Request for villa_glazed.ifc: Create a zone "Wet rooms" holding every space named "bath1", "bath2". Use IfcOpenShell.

First a look at what the model holds.

```python
import ifcopenshell

model = ifcopenshell.open("villa_glazed.ifc")
print(model.schema)
seen = {}
for space in model.by_type("IfcSpace"):
    seen[space.LongName] = seen.get(space.LongName, 0) + 1
for name, count in sorted(seen.items(), key=str):
    print(count, "x", name)
print("zones:", [z.Name for z in model.by_type("IfcZone")][:20])
```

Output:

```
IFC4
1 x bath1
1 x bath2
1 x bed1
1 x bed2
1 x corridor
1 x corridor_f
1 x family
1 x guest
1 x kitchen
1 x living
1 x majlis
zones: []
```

```python
import ifcopenshell
import ifcopenshell.api.group
import ifcopenshell.api.root

model = ifcopenshell.open("villa_glazed.ifc")

names = {"bath1", "bath2"}
spaces = [s for s in model.by_type("IfcSpace") if s.LongName in names]

zone = ifcopenshell.api.root.create_entity(model, ifc_class="IfcZone", name="Wet rooms")
ifcopenshell.api.group.assign_group(model, products=spaces, group=zone)
print(len(spaces), "spaces in", zone.Name)

model.write("villa_glazed_edited.ifc")
```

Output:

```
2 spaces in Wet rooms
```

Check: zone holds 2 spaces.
